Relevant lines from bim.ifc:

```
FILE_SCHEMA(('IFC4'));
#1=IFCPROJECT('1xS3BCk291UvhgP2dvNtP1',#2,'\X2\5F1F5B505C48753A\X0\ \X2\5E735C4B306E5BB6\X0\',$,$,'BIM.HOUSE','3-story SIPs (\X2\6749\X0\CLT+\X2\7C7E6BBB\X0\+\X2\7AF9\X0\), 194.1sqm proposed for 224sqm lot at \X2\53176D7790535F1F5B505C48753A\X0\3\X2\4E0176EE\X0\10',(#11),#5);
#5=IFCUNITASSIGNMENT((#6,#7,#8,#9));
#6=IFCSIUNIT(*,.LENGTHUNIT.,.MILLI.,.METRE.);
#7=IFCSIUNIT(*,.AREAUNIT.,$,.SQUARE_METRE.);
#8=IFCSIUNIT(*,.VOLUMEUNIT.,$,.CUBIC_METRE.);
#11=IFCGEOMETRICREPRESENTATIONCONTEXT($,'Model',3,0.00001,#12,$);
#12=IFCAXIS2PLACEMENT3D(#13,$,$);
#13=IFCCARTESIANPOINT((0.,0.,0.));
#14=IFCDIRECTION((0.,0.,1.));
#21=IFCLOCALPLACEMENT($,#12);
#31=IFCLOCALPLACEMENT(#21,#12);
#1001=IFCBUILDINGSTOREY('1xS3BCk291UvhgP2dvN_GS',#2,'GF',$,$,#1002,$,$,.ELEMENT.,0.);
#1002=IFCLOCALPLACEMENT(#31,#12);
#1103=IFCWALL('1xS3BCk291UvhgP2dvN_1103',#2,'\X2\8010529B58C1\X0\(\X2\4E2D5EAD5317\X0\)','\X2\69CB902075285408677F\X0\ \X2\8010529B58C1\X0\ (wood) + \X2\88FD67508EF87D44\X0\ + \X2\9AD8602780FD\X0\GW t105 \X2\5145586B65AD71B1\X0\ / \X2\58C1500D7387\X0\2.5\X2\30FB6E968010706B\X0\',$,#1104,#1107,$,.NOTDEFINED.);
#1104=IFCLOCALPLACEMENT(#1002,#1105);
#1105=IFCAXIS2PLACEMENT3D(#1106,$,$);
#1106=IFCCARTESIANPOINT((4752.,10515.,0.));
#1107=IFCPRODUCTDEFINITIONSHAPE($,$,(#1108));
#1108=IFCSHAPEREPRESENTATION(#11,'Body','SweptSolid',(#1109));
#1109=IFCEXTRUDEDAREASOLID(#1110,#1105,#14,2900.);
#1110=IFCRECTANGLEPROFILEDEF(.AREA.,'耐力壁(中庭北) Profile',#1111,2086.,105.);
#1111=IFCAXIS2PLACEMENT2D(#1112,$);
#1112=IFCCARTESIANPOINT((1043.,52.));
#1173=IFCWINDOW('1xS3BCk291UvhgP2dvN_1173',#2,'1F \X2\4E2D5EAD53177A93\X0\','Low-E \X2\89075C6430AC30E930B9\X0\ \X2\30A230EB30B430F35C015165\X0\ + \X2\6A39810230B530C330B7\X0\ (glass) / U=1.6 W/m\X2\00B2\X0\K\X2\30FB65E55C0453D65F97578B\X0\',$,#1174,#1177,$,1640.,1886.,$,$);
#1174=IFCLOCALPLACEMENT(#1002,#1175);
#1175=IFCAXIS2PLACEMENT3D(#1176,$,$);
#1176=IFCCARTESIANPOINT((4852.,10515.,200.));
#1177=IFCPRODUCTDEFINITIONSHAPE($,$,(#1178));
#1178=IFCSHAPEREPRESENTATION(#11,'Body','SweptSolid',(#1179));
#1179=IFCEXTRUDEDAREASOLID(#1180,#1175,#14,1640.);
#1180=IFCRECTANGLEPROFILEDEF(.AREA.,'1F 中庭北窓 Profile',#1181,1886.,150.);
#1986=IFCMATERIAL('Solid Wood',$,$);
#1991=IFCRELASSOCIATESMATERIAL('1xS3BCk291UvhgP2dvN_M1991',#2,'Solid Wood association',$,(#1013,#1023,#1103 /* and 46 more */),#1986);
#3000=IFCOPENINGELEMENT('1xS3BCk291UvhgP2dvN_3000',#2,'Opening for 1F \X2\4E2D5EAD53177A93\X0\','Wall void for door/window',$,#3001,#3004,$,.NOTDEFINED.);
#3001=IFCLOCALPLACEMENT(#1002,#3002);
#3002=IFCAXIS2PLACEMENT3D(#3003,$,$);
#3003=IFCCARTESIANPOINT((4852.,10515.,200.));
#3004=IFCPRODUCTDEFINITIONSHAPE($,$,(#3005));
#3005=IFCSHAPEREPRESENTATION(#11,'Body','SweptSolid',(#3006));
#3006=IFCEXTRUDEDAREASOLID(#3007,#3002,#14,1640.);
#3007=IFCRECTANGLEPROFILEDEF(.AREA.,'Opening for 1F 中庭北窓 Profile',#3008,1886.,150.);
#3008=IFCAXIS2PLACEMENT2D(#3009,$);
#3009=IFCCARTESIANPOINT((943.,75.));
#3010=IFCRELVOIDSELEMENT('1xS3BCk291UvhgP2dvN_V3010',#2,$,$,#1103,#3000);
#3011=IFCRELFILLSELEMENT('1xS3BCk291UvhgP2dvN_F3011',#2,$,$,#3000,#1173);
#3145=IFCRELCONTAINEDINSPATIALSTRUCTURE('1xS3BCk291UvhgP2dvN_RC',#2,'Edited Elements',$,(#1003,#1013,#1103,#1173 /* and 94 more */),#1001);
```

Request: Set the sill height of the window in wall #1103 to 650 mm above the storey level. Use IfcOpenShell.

```python
import numpy as np
import ifcopenshell
import ifcopenshell.api.geometry
import ifcopenshell.geom
import ifcopenshell.util.element
import ifcopenshell.util.placement
import ifcopenshell.util.shape
import ifcopenshell.util.unit

model = ifcopenshell.open("bim.ifc")
unit_scale = ifcopenshell.util.unit.calculate_unit_scale(model)

window = model.by_guid("1xS3BCk291UvhgP2dvN_1173")
opening = window.FillsVoids[0].RelatingOpeningElement
storey = ifcopenshell.util.element.get_container(window, ifc_class="IfcBuildingStorey")
level = ifcopenshell.util.placement.get_local_placement(storey.ObjectPlacement)[2, 3]

# The opening's origin need not be at the sill, so measure its lowest point.
shape = ifcopenshell.geom.create_shape(ifcopenshell.geom.settings(), opening)
bottom = ifcopenshell.util.shape.get_shape_bottom_elevation(shape, shape.geometry) / unit_scale
dz = level + 650.0 - bottom

shift = np.array([0.0, 0.0, dz])
# The window is not placed relative to its opening, so move both.
for product in (opening, window):
    matrix = ifcopenshell.util.placement.get_local_placement(product.ObjectPlacement)
    matrix[:3, 3] += shift
    ifcopenshell.api.geometry.edit_object_placement(model, product=product, matrix=matrix, is_si=False)

print(f"moved by {dz * unit_scale:+.3f} m")

model.write("bim-out.ifc")
```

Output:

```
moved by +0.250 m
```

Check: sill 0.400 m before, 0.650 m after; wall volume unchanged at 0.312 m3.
